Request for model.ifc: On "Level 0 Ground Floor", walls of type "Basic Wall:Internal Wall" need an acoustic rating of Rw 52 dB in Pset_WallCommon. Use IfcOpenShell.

First a look at what the model holds.

```python
import ifcopenshell
import ifcopenshell.util.element

model = ifcopenshell.open("model.ifc")
print(model.schema)
storey = next(s for s in model.by_type("IfcBuildingStorey") if s.Name == "Level 0 Ground Floor")
walls = [e for e in ifcopenshell.util.element.get_decomposition(storey) if e.is_a("IfcWall")]
seen = {}
for e in walls:
    element_type = ifcopenshell.util.element.get_type(e)
    key = (element_type.Name if element_type != e and element_type else None, ifcopenshell.util.element.get_pset(e, "Pset_WallCommon", "AcousticRating"))
    seen[key] = seen.get(key, 0) + 1
for (name, value), count in sorted(seen.items(), key=str):
    print(count, "x", name, "|", value)
```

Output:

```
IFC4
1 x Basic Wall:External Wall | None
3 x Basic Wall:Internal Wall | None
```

```python
import ifcopenshell
import ifcopenshell.api.pset
import ifcopenshell.util.element

model = ifcopenshell.open("model.ifc")

storey = next(s for s in model.by_type("IfcBuildingStorey") if s.Name == "Level 0 Ground Floor")
walls = [e for e in ifcopenshell.util.element.get_decomposition(storey) if e.is_a("IfcWall")]

count = 0
for e in walls:
    element_type = ifcopenshell.util.element.get_type(e)
    if element_type in (None, e) or element_type.Name != "Basic Wall:Internal Wall":
        continue
    # add_pset returns the element's existing set when there is one.
    pset = ifcopenshell.api.pset.add_pset(model, product=e, name="Pset_WallCommon")
    ifcopenshell.api.pset.edit_pset(model, pset=pset, properties={"AcousticRating": "Rw 52 dB"})
    count += 1

print(count, "walls updated")

model.write("model_updated.ifc")
```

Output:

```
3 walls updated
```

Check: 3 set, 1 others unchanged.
